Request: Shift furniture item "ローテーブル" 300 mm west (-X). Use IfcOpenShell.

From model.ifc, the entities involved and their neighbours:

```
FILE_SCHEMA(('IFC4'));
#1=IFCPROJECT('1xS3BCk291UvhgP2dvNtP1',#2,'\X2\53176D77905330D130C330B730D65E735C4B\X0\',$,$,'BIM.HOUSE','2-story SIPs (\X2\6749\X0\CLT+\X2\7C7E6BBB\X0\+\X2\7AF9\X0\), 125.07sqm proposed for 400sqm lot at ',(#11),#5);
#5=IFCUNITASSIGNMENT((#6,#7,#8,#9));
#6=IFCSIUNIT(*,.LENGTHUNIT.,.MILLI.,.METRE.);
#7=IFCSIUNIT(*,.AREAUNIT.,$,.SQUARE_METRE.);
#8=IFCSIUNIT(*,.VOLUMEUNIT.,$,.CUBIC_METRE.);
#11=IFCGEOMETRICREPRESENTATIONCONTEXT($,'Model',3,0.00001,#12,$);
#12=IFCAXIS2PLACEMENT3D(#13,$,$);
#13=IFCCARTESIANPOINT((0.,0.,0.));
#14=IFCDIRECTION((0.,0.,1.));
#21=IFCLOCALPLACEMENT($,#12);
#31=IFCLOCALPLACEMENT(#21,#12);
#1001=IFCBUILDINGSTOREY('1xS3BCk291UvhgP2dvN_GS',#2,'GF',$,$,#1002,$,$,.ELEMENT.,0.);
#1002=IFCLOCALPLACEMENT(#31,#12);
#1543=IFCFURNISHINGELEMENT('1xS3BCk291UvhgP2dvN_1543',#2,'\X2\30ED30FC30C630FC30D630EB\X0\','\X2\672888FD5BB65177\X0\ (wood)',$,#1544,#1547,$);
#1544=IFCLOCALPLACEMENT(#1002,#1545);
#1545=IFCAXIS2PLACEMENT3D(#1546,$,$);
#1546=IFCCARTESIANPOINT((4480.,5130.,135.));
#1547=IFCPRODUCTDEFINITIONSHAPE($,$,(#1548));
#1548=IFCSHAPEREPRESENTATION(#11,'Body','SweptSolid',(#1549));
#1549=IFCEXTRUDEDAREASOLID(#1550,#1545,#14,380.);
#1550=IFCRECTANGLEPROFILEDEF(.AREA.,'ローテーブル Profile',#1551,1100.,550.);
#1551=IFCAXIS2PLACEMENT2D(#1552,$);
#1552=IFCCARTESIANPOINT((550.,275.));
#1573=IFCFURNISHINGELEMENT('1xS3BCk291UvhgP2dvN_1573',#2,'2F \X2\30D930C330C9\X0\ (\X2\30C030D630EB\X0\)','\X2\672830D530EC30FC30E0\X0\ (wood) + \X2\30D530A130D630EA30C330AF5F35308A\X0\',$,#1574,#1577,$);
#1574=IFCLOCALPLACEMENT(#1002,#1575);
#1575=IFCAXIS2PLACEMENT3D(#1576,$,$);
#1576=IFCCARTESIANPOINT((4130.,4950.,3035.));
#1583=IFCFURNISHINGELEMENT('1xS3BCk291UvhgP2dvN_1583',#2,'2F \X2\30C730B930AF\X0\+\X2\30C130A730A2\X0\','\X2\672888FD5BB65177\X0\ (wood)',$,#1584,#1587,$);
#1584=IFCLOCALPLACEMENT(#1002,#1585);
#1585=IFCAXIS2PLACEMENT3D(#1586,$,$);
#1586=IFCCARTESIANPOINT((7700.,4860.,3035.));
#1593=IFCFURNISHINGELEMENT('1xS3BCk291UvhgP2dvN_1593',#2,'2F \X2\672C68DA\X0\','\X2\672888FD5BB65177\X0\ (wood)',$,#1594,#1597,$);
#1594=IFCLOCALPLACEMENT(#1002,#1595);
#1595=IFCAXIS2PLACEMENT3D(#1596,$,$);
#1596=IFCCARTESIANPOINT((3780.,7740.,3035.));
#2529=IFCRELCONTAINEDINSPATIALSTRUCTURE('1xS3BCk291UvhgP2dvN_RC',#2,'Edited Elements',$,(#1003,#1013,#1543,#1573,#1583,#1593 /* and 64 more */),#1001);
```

```python
import ifcopenshell
import ifcopenshell.api.geometry
import ifcopenshell.util.placement

model = ifcopenshell.open("model.ifc")

item = model.by_id(1543)
matrix = ifcopenshell.util.placement.get_local_placement(item.ObjectPlacement)
matrix[0, 3] -= 300.0
ifcopenshell.api.geometry.edit_object_placement(model, product=item, matrix=matrix, is_si=False)

print(ifcopenshell.util.placement.get_local_placement(item.ObjectPlacement).round(3) + 0.0)

model.write("model_v2.ifc")
```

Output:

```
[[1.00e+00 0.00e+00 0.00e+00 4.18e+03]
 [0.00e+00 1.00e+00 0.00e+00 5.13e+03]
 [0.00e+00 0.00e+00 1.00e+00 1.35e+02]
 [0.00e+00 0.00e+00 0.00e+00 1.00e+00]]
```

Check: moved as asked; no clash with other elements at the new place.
